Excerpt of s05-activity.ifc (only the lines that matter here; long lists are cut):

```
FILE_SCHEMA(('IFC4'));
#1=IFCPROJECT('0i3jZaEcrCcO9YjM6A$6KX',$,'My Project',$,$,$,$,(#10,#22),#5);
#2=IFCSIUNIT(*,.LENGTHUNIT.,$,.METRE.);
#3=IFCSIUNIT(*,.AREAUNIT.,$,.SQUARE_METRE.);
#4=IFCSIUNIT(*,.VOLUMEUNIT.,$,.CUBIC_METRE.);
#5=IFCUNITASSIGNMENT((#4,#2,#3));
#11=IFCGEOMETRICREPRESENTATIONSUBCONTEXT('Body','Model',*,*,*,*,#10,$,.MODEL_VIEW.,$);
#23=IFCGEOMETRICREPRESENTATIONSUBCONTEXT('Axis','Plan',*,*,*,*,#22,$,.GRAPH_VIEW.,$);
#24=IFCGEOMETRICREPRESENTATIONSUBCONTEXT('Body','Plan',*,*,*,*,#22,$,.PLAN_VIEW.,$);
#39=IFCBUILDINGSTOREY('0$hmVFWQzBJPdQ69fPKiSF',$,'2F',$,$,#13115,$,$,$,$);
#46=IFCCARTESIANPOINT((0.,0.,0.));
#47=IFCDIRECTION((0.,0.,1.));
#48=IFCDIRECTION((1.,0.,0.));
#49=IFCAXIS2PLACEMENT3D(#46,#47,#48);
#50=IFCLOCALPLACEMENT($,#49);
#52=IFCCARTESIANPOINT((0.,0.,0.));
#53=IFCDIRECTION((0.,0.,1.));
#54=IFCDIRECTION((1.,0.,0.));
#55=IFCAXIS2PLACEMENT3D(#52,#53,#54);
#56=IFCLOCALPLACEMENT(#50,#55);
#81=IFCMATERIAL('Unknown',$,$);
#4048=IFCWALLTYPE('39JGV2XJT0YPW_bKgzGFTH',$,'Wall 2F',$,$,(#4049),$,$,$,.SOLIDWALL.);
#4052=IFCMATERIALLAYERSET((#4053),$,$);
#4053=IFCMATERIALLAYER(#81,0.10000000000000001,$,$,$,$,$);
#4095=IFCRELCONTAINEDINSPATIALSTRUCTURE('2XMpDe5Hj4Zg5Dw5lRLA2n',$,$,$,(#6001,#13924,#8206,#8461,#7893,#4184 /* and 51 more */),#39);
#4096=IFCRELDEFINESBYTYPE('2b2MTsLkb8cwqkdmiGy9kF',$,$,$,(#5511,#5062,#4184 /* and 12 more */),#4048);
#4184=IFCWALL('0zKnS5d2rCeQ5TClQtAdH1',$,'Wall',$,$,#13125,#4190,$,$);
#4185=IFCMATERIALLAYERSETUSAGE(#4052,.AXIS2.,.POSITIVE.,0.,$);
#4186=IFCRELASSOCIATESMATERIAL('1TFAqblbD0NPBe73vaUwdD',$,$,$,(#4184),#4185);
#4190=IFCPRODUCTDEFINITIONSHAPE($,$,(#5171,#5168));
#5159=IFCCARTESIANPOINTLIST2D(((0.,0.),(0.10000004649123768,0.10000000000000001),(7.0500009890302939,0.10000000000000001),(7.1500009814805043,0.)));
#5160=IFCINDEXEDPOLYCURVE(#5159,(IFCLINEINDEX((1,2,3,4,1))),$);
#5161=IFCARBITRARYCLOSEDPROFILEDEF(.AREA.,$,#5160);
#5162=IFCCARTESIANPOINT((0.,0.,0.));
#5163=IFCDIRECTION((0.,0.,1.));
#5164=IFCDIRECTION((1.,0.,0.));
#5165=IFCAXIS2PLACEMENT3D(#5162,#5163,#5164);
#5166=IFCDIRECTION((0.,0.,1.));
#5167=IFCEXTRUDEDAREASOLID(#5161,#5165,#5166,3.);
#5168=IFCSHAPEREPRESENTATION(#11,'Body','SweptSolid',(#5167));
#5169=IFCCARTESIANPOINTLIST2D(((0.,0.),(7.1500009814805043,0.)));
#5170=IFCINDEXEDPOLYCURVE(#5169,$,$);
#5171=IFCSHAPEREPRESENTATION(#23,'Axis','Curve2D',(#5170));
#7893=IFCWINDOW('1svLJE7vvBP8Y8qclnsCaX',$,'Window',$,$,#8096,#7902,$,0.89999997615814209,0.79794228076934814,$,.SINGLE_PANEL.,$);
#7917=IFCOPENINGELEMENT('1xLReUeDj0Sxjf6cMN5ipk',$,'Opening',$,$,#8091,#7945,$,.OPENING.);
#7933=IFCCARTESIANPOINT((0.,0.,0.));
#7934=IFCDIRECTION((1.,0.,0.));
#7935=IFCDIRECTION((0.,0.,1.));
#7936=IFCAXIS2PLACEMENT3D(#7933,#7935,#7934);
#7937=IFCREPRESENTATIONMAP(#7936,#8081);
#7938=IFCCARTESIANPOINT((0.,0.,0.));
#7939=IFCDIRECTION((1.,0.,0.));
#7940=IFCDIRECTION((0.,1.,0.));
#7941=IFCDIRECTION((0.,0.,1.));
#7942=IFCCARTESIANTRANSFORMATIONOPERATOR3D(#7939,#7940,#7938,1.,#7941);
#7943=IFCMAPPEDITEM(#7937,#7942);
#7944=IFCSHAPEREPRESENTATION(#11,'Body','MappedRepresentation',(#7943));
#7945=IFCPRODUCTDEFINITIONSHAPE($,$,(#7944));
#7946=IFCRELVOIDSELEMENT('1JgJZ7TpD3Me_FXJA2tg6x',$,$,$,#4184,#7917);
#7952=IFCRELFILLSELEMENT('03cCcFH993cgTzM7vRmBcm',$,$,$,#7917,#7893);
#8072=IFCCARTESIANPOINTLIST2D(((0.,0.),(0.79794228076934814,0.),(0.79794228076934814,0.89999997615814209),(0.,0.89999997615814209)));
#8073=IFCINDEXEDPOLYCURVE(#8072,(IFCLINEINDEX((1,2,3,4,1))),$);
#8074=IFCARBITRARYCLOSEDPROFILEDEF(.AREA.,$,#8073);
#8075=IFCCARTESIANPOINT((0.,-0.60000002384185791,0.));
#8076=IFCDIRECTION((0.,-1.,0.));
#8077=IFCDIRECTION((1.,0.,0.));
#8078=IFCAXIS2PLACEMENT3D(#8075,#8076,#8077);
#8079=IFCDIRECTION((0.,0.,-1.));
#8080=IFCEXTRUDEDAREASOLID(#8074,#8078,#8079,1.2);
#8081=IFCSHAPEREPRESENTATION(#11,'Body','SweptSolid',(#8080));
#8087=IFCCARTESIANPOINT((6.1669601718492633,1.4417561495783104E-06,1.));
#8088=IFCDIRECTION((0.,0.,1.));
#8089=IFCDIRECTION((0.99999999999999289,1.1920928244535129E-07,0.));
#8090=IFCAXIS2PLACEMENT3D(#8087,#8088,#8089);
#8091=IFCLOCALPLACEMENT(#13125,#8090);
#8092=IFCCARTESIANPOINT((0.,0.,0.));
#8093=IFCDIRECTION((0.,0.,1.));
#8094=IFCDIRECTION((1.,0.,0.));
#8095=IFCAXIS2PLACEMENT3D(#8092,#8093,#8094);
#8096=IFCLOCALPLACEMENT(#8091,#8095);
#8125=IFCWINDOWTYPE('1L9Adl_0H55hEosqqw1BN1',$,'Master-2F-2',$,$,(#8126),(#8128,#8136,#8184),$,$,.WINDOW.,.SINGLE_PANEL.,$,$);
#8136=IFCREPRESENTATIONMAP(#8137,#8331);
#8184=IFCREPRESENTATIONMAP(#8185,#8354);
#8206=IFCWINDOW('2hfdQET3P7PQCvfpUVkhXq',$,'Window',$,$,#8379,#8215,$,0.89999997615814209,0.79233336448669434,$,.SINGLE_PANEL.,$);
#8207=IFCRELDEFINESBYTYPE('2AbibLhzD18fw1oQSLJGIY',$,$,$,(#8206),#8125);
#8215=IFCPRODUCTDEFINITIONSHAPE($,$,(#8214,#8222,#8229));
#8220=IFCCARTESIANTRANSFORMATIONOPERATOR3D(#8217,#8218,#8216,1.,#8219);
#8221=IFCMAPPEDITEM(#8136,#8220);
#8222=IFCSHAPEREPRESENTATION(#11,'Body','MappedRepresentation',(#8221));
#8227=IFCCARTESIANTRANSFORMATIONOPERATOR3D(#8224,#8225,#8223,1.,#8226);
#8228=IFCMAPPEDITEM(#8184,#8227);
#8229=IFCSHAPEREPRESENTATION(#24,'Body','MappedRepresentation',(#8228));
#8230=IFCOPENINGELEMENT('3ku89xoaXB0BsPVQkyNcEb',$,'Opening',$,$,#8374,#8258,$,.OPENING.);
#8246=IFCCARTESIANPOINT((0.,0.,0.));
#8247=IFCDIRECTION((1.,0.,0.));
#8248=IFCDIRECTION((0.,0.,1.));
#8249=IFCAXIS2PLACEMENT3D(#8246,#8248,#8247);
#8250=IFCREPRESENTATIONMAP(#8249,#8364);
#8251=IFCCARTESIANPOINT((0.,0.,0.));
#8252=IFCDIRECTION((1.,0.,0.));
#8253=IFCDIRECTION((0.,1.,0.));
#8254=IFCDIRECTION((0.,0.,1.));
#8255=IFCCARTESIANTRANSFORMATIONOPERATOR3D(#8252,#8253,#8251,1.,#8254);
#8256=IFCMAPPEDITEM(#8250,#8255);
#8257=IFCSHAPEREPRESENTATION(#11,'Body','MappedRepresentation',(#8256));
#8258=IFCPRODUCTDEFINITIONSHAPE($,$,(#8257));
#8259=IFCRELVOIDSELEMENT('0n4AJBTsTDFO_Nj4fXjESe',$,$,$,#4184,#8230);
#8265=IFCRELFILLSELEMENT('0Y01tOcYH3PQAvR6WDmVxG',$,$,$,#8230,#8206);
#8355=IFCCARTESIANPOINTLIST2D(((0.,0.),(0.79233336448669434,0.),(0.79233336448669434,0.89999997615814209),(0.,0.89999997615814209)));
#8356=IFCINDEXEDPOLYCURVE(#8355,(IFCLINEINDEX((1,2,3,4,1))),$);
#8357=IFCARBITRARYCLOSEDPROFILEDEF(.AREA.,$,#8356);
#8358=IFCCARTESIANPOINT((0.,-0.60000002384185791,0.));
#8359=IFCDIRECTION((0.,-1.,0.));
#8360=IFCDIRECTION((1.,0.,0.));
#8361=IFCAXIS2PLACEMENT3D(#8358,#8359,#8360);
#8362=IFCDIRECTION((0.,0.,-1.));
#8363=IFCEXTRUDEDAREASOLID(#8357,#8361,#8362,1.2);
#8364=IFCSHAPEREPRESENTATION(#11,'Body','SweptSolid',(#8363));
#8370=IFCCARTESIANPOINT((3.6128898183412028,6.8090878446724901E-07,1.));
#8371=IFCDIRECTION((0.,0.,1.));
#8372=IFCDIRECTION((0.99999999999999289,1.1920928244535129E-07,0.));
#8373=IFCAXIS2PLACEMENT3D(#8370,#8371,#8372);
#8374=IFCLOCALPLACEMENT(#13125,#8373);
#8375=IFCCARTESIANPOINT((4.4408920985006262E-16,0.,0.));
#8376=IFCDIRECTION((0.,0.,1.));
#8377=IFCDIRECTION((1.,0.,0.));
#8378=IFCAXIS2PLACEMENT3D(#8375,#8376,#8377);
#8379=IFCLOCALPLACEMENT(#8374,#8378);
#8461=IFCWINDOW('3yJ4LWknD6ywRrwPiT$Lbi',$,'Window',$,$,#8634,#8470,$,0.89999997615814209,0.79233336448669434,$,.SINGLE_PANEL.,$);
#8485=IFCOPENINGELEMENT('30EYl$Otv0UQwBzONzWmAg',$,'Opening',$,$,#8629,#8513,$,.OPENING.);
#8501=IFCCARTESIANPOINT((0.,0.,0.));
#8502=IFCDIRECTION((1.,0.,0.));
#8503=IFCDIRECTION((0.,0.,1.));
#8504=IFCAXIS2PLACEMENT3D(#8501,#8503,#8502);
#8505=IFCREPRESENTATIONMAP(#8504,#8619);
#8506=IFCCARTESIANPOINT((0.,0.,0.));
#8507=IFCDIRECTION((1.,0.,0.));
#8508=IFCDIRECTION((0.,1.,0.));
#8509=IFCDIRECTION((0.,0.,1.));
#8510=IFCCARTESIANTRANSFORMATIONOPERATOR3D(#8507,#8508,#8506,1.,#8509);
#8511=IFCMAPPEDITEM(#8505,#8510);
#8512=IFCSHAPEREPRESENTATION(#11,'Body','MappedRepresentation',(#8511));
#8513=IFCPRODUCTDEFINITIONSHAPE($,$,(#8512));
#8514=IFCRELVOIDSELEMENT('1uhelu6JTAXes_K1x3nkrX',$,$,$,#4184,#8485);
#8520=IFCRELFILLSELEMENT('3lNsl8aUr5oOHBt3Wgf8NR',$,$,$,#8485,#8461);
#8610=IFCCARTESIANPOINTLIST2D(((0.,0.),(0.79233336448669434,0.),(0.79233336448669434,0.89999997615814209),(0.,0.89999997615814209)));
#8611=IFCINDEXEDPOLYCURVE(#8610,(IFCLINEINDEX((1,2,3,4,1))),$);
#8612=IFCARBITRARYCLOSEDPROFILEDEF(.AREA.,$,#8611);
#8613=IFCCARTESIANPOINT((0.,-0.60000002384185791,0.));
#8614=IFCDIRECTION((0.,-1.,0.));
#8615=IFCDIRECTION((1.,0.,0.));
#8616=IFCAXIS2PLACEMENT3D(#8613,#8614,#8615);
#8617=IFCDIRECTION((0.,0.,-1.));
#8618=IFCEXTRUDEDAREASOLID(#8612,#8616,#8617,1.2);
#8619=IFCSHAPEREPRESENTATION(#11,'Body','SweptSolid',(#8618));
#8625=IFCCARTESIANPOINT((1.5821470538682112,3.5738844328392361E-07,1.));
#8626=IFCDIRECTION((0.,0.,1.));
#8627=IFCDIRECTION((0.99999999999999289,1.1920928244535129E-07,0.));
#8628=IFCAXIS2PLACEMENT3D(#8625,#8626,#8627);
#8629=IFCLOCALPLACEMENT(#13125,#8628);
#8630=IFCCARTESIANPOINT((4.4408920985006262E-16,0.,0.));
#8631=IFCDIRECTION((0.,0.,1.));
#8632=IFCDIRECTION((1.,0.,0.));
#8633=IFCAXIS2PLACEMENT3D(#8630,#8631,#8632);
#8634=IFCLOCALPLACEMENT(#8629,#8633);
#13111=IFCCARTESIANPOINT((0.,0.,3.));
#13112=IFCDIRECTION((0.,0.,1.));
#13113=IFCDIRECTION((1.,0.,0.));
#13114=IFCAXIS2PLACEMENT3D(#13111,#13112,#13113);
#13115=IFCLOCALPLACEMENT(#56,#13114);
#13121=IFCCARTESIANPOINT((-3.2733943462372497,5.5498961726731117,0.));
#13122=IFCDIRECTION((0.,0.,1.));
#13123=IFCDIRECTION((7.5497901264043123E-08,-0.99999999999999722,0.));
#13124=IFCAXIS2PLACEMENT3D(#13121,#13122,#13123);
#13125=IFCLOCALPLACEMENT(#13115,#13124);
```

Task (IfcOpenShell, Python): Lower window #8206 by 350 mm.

```python
import numpy as np
import ifcopenshell
import ifcopenshell.api.geometry
import ifcopenshell.util.placement
import ifcopenshell.util.unit

model = ifcopenshell.open("s05-activity.ifc")
unit_scale = ifcopenshell.util.unit.calculate_unit_scale(model)

window = model.by_guid("2hfdQET3P7PQCvfpUVkhXq")
opening = window.FillsVoids[0].RelatingOpeningElement
dz = -0.35 / unit_scale

shift = np.array([0.0, 0.0, dz])
# The window is placed relative to its opening, so it follows when the opening moves.
matrix = ifcopenshell.util.placement.get_local_placement(opening.ObjectPlacement)
matrix[:3, 3] += shift
ifcopenshell.api.geometry.edit_object_placement(
    model, product=opening, matrix=matrix, is_si=False, should_transform_children=True
)

print(f"moved by {dz * unit_scale:+.3f} m")

model.write("s05-activity_updated.ifc")
```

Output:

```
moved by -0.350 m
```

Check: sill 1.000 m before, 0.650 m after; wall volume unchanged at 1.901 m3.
